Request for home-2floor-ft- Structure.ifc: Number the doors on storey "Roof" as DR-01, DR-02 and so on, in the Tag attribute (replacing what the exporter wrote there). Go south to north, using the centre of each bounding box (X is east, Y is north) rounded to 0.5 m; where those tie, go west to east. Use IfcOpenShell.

First a look at what the model holds.

```python
import ifcopenshell
import ifcopenshell.util.element
import ifcopenshell.util.placement

model = ifcopenshell.open("home-2floor-ft- Structure.ifc")
print(model.schema)
storey = next(s for s in model.by_type("IfcBuildingStorey") if s.Name == "Roof")
doors = [e for e in ifcopenshell.util.element.get_decomposition(storey) if e.is_a("IfcDoor")]
for e in sorted(doors, key=lambda e: e.id()):
    origin = ifcopenshell.util.placement.get_local_placement(e.ObjectPlacement)[:3, 3]
    print(e.id(), e.Tag, e.Name, origin.round(2) + 0.0, sep=" | ")
```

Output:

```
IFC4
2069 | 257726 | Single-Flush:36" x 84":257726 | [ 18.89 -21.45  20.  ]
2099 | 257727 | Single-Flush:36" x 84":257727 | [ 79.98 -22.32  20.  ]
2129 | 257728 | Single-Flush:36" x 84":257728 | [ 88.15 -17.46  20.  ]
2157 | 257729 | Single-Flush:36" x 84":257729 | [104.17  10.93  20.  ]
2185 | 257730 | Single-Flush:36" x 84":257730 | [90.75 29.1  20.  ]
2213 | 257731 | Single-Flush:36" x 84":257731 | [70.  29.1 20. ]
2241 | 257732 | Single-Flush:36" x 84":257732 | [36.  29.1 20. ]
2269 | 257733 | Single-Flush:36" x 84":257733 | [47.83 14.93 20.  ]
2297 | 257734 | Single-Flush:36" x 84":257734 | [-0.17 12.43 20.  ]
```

```python
import ifcopenshell
import ifcopenshell.geom
import ifcopenshell.util.element
import ifcopenshell.util.shape

model = ifcopenshell.open("home-2floor-ft- Structure.ifc")
settings = ifcopenshell.geom.settings()
settings.set("use-world-coords", True)


def centre(element):
    shape = ifcopenshell.geom.create_shape(settings, element)
    return ifcopenshell.util.shape.get_bbox_centroid(shape.geometry)


storey = next(s for s in model.by_type("IfcBuildingStorey") if s.Name == "Roof")
doors = [e for e in ifcopenshell.util.element.get_decomposition(storey) if e.is_a("IfcDoor")]

# Insertion points can sit at a corner or the storey origin, so sort by the geometry (in metres).
centres = {e: centre(e) for e in doors}
doors.sort(key=lambda e: (round(centres[e][1] / 0.5), centres[e][0]))

for i, e in enumerate(doors, start=1):
    number = f"DR-{i:02d}"
    e.Tag = number
    print(e.id(), number)

model.write("home-2floor-ft- Structure_rev.ifc")
```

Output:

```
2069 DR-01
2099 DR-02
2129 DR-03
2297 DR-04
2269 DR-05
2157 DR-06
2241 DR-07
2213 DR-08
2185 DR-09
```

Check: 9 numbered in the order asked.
